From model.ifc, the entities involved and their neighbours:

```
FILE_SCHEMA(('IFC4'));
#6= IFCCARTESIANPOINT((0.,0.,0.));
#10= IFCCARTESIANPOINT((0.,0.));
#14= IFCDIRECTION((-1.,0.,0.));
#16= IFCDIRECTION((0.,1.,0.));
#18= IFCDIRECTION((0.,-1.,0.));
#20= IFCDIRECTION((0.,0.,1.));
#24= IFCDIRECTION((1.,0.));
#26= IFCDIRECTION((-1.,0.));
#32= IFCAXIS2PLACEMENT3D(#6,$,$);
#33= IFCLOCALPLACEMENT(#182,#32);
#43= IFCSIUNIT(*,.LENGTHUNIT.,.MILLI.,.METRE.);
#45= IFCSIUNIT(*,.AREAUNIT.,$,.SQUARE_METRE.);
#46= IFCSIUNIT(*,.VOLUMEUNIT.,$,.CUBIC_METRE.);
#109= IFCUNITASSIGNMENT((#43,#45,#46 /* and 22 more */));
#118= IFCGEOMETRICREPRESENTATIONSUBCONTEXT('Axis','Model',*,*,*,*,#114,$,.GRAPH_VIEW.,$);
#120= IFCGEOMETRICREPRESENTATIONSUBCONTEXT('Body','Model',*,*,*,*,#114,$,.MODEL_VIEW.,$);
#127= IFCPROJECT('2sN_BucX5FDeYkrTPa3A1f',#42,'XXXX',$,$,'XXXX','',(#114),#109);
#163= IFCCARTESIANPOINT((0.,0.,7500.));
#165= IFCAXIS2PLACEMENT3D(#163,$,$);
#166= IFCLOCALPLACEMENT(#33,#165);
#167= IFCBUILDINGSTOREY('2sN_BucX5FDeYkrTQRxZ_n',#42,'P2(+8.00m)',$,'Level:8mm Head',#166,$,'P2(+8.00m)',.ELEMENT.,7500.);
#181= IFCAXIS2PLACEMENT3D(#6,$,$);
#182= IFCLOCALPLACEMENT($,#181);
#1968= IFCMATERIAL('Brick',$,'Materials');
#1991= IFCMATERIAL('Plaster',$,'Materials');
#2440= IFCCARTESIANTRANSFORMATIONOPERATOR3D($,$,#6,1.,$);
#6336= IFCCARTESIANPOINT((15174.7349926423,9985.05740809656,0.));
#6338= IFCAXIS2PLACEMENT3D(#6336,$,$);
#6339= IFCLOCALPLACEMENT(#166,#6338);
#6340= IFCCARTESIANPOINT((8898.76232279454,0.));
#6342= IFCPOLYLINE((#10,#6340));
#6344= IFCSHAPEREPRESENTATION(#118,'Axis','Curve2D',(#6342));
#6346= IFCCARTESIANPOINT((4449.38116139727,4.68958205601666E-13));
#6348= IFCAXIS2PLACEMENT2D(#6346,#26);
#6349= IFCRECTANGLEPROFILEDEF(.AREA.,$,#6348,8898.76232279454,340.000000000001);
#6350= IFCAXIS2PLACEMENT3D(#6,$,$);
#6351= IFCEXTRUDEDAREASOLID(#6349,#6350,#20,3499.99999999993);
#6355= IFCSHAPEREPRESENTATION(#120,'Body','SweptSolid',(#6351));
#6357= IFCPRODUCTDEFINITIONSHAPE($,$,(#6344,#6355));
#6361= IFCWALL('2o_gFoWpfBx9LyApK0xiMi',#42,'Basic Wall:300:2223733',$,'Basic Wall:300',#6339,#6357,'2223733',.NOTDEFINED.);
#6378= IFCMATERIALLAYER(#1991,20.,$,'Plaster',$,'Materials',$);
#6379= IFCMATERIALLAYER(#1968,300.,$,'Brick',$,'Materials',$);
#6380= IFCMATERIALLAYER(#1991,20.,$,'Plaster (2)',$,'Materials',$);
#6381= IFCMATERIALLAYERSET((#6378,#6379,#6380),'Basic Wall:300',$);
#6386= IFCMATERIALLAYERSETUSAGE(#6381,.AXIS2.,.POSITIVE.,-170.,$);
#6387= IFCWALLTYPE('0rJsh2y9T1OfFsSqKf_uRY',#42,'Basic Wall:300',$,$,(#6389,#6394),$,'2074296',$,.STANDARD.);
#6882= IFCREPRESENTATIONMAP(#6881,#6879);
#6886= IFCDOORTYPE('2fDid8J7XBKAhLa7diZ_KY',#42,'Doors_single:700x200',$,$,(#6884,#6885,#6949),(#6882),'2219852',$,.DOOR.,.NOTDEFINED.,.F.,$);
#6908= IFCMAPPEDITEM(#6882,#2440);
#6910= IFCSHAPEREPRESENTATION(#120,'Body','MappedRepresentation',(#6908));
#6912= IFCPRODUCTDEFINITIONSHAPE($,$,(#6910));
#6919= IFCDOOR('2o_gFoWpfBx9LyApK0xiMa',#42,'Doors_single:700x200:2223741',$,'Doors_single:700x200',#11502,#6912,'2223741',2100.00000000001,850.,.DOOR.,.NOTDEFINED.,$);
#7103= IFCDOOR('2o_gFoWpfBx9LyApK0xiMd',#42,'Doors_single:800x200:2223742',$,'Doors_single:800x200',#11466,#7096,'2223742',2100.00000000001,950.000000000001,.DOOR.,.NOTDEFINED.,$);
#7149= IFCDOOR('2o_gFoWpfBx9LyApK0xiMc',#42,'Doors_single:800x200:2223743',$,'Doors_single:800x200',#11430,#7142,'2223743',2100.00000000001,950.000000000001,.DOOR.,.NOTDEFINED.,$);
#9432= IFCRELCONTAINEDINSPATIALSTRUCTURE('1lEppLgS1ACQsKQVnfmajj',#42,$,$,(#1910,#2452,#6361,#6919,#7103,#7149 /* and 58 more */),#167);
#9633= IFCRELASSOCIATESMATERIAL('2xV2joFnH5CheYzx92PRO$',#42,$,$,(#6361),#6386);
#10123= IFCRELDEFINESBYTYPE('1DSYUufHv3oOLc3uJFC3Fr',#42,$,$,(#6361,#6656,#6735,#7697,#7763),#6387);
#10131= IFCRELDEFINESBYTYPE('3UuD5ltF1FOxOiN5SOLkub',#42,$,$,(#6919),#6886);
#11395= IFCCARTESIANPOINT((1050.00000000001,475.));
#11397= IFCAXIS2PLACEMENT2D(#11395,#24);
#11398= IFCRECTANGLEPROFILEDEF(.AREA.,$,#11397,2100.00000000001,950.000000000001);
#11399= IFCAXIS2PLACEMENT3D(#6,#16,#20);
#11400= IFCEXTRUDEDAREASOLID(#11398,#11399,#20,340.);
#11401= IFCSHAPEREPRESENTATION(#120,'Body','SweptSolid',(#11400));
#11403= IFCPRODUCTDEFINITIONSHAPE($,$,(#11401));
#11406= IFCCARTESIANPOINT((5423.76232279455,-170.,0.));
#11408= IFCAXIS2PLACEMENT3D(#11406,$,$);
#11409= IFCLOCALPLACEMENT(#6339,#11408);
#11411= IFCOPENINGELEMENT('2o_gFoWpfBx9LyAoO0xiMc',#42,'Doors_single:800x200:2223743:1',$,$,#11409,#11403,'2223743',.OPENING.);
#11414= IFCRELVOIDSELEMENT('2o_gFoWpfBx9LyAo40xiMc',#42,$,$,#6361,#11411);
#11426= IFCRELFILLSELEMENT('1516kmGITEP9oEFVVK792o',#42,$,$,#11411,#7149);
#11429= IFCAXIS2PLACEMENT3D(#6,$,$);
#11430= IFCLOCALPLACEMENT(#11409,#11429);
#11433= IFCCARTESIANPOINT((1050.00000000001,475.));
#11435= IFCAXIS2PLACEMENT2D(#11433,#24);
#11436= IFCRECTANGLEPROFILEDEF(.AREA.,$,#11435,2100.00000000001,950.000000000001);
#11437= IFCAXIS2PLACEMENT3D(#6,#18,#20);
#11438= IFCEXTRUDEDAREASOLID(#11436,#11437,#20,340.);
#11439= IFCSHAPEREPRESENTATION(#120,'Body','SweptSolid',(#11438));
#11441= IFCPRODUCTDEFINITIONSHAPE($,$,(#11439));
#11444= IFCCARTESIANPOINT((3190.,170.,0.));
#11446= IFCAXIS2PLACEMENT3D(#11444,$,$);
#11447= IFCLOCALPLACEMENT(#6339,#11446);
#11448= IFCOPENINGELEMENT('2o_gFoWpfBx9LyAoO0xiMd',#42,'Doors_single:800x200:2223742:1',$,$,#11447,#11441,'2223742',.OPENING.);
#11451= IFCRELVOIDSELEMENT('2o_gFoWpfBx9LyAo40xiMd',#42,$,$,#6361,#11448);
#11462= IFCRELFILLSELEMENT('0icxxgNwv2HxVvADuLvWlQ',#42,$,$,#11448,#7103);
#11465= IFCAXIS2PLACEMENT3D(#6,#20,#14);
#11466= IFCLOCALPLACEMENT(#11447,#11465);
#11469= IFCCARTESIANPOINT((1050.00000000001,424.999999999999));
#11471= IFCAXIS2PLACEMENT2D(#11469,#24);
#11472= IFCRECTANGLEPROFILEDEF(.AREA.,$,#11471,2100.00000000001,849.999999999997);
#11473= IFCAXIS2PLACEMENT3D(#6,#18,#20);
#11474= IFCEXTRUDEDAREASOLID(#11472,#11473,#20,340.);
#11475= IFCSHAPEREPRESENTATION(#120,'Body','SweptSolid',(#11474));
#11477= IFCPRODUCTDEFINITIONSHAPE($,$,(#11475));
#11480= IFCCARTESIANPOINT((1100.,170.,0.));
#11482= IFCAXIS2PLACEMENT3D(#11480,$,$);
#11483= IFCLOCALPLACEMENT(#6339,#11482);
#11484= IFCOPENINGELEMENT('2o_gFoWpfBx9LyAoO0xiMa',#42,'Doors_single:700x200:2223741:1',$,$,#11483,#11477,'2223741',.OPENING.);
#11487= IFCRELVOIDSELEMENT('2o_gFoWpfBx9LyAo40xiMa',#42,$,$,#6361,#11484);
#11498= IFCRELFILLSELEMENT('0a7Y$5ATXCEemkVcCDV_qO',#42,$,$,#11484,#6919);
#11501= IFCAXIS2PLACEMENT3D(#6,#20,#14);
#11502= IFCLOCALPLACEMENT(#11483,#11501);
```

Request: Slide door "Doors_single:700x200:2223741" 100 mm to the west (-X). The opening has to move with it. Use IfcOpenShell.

```python
import ifcopenshell
import ifcopenshell.api.geometry
import ifcopenshell.util.placement
import ifcopenshell.util.unit

model = ifcopenshell.open("model.ifc")
unit_scale = ifcopenshell.util.unit.calculate_unit_scale(model)

door = model.by_guid("2o_gFoWpfBx9LyApK0xiMa")
opening = door.FillsVoids[0].RelatingOpeningElement
wall = opening.VoidsElements[0].RelatingBuildingElement

wall_matrix = ifcopenshell.util.placement.get_local_placement(wall.ObjectPlacement)
shift = wall_matrix[:3, 0] * -0.1 / unit_scale
before = ifcopenshell.util.placement.get_local_placement(door.ObjectPlacement)[:3, 3].copy()

# The door is placed relative to its opening, so it follows when the opening moves.
matrix = ifcopenshell.util.placement.get_local_placement(opening.ObjectPlacement)
matrix[:3, 3] += shift
ifcopenshell.api.geometry.edit_object_placement(
    model, product=opening, matrix=matrix, is_si=False, should_transform_children=True
)

after = ifcopenshell.util.placement.get_local_placement(door.ObjectPlacement)[:3, 3]
print("door moved by", (after - before).round(3) + 0.0)

model.write("model_v2.ifc")
```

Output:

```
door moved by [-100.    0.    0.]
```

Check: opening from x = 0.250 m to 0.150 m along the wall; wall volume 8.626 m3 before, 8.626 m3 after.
